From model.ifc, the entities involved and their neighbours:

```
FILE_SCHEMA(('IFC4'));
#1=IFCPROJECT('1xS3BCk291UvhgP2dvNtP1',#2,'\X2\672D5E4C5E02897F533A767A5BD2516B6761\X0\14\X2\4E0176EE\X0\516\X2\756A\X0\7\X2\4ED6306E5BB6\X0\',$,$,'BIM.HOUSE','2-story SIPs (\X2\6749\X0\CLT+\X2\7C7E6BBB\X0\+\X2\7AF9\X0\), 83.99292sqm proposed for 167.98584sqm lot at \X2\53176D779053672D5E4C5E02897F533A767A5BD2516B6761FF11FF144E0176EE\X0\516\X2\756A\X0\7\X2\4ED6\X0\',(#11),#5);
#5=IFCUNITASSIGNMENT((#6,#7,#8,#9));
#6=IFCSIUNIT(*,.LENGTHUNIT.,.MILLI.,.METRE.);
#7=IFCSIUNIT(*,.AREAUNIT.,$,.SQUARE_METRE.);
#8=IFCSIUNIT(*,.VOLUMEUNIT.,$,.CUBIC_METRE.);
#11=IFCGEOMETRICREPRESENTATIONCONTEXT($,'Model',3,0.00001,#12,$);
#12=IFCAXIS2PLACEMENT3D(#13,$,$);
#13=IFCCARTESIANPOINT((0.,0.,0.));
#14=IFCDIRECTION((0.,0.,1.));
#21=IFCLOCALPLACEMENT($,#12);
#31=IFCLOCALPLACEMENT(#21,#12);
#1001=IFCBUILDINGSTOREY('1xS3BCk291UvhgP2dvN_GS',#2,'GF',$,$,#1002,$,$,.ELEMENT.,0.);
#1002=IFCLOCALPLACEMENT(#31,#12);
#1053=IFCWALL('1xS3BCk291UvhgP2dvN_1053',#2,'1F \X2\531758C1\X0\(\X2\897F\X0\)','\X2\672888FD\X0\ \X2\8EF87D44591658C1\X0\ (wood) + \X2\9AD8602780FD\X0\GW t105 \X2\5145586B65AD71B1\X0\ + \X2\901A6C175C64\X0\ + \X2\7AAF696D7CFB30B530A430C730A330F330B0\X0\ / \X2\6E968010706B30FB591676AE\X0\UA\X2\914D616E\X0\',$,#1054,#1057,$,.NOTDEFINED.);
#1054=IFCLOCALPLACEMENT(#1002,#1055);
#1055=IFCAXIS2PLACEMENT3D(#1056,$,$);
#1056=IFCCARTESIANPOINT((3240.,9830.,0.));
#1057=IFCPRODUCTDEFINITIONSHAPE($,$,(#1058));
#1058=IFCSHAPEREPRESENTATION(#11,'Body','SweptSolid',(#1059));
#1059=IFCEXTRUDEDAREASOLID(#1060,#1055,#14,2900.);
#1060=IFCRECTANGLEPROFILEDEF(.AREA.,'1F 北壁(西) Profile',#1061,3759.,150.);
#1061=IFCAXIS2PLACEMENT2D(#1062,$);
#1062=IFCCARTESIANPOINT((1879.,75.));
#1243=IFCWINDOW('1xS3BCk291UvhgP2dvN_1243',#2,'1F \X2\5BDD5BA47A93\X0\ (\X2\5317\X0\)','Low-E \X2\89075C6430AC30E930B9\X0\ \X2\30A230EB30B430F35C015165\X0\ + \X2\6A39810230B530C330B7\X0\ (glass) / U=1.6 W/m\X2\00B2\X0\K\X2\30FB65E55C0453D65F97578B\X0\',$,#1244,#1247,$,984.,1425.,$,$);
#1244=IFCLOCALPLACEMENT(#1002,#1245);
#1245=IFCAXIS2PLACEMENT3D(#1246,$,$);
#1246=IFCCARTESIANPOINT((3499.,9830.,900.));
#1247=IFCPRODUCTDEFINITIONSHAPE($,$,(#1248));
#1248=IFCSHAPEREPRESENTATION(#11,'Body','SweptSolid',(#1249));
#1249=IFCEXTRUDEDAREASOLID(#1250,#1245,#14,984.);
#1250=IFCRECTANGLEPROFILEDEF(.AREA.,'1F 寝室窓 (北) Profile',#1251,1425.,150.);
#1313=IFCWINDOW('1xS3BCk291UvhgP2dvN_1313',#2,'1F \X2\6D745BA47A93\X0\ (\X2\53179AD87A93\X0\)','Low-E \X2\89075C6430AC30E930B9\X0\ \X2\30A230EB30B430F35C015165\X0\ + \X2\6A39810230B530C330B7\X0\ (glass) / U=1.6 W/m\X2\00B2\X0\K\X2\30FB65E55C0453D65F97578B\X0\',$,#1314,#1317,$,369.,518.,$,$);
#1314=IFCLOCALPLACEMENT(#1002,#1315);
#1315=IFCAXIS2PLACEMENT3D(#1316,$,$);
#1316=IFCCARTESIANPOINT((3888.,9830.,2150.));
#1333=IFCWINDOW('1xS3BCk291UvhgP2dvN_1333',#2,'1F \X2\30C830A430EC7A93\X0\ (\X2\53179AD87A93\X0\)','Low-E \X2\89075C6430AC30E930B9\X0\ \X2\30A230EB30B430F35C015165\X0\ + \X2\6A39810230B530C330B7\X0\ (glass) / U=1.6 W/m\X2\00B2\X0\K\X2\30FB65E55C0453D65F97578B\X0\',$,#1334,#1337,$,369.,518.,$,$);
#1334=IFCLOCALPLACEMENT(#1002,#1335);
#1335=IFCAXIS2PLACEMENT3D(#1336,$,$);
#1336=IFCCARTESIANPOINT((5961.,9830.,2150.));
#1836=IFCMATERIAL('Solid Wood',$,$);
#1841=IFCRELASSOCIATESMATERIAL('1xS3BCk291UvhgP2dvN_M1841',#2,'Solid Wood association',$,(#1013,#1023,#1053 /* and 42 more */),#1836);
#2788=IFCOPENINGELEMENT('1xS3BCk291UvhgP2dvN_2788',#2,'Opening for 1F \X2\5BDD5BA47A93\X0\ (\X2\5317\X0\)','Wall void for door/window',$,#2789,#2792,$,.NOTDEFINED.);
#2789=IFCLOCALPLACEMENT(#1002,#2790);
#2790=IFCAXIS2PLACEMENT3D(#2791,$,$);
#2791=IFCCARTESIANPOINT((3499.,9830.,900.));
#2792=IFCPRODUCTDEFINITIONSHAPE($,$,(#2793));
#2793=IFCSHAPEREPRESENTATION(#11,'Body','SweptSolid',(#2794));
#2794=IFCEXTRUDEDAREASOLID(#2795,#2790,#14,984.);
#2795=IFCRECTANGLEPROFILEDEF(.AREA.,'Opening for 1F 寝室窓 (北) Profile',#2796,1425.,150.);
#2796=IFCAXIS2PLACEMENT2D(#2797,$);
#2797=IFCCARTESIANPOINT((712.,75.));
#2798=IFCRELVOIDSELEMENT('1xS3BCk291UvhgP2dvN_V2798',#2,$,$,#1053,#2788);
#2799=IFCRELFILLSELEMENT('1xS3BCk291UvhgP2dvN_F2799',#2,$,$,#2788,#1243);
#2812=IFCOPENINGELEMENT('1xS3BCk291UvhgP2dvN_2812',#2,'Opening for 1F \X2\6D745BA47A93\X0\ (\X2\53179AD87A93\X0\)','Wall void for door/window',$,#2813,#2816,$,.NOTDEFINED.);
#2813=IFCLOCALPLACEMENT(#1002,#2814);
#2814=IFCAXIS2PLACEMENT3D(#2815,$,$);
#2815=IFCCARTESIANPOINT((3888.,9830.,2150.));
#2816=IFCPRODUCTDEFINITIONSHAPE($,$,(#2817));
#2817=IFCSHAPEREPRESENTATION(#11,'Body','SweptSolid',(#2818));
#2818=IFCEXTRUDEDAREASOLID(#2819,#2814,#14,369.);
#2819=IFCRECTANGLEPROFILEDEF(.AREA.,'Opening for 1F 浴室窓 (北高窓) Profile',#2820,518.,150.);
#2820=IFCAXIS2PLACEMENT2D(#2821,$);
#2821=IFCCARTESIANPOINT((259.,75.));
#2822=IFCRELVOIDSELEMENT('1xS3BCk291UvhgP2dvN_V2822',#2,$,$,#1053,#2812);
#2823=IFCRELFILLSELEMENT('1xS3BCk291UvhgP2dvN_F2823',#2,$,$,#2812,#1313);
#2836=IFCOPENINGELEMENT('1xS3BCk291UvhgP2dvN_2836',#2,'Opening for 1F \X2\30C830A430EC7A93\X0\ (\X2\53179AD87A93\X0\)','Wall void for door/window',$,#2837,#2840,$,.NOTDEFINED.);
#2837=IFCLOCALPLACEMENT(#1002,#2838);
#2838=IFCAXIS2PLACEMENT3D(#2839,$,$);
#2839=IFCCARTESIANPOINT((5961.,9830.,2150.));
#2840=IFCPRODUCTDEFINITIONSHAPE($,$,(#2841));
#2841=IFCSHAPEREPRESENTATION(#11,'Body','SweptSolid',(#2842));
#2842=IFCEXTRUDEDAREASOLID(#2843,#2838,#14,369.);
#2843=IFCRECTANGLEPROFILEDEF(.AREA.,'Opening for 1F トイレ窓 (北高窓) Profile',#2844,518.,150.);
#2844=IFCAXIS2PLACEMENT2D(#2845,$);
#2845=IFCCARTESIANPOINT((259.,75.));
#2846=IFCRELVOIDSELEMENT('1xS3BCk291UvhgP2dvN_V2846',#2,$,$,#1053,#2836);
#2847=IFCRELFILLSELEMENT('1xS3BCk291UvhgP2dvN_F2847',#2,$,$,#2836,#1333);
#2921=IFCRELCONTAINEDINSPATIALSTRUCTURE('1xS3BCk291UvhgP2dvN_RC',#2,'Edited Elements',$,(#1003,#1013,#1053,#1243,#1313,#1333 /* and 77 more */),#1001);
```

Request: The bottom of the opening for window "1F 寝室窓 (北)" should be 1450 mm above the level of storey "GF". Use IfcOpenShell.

```python
import numpy as np
import ifcopenshell
import ifcopenshell.api.geometry
import ifcopenshell.geom
import ifcopenshell.util.element
import ifcopenshell.util.placement
import ifcopenshell.util.shape
import ifcopenshell.util.unit

model = ifcopenshell.open("model.ifc")
unit_scale = ifcopenshell.util.unit.calculate_unit_scale(model)

window = model.by_guid("1xS3BCk291UvhgP2dvN_1243")
opening = window.FillsVoids[0].RelatingOpeningElement
storey = ifcopenshell.util.element.get_container(window, ifc_class="IfcBuildingStorey")
level = ifcopenshell.util.placement.get_local_placement(storey.ObjectPlacement)[2, 3]

# The opening's origin need not be at the sill, so measure its lowest point.
shape = ifcopenshell.geom.create_shape(ifcopenshell.geom.settings(), opening)
bottom = ifcopenshell.util.shape.get_shape_bottom_elevation(shape, shape.geometry) / unit_scale
dz = level + 1450.0 - bottom

shift = np.array([0.0, 0.0, dz])
# The window is not placed relative to its opening, so move both.
for product in (opening, window):
    matrix = ifcopenshell.util.placement.get_local_placement(product.ObjectPlacement)
    matrix[:3, 3] += shift
    ifcopenshell.api.geometry.edit_object_placement(model, product=product, matrix=matrix, is_si=False)

print(f"moved by {dz * unit_scale:+.3f} m")

model.write("model_rev.ifc")
```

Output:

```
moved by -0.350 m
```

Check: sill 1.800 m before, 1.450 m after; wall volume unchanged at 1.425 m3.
